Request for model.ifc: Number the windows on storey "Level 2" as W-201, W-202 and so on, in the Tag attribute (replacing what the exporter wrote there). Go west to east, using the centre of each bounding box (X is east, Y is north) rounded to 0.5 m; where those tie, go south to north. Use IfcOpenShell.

First a look at what the model holds.

```python
import ifcopenshell
import ifcopenshell.util.element
import ifcopenshell.util.placement

model = ifcopenshell.open("model.ifc")
print(model.schema)
storey = next(s for s in model.by_type("IfcBuildingStorey") if s.Name == "Level 2")
windows = [e for e in ifcopenshell.util.element.get_decomposition(storey) if e.is_a("IfcWindow")]
for e in sorted(windows, key=lambda e: e.id()):
    origin = ifcopenshell.util.placement.get_local_placement(e.ObjectPlacement)[:3, 3]
    print(e.id(), e.Tag, e.Name, origin.round(2) + 0.0, sep=" | ")
```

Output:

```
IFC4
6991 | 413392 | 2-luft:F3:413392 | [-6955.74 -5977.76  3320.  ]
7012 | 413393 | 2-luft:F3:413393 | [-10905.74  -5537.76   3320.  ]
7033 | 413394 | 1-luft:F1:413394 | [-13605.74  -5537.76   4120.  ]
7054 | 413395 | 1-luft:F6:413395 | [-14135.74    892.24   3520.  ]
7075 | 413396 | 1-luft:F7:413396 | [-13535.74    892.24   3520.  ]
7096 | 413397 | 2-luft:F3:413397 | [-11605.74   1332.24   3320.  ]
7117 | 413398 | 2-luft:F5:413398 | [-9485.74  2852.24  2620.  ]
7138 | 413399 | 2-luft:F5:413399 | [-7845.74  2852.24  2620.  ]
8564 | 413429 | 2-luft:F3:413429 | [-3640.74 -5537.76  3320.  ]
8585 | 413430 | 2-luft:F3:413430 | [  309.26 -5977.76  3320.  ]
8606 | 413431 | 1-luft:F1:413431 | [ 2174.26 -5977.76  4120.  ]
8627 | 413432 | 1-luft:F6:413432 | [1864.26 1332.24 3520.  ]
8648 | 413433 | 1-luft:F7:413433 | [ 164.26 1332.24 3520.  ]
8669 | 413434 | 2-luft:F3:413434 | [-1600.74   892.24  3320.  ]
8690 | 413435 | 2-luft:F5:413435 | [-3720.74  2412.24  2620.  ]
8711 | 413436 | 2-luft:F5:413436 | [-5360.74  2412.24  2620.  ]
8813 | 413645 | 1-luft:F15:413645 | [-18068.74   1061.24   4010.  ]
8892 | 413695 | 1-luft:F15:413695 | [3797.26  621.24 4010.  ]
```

```python
import ifcopenshell
import ifcopenshell.geom
import ifcopenshell.util.element
import ifcopenshell.util.shape

model = ifcopenshell.open("model.ifc")
settings = ifcopenshell.geom.settings()
settings.set("use-world-coords", True)


def centre(element):
    shape = ifcopenshell.geom.create_shape(settings, element)
    return ifcopenshell.util.shape.get_bbox_centroid(shape.geometry)


storey = next(s for s in model.by_type("IfcBuildingStorey") if s.Name == "Level 2")
windows = [e for e in ifcopenshell.util.element.get_decomposition(storey) if e.is_a("IfcWindow")]

# Insertion points can sit at a corner or the storey origin, so sort by the geometry (in metres).
centres = {e: centre(e) for e in windows}
windows.sort(key=lambda e: (round(centres[e][0] / 0.5), centres[e][1]))

for i, e in enumerate(windows, start=1):
    number = f"W-2{i:02d}"
    e.Tag = number
    print(e.id(), number)

model.write("model_updated.ifc")
```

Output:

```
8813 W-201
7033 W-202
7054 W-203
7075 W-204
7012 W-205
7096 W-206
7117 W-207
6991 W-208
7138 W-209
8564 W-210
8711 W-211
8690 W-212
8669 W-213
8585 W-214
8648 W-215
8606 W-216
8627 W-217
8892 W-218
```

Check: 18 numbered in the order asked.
